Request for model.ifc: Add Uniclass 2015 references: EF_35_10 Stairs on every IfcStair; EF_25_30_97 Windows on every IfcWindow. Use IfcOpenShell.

First a look at what the model holds.

```python
import ifcopenshell

model = ifcopenshell.open("model.ifc")
print(model.schema)
print("classifications:", [c.Name for c in model.by_type("IfcClassification")])
for ifc_class in ("IfcDoor", "IfcRoof", "IfcStair", "IfcWall", "IfcWindow"):
    print(ifc_class, len(model.by_type(ifc_class)))
```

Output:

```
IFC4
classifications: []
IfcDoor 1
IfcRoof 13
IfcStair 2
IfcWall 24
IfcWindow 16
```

```python
import ifcopenshell
import ifcopenshell.api.classification

model = ifcopenshell.open("model.ifc")

system = ifcopenshell.api.classification.add_classification(model, classification="Uniclass 2015")

codes = {
    "IfcStair": ("EF_35_10", "Stairs"),
    "IfcWindow": ("EF_25_30_97", "Windows"),
}
for ifc_class, (code, name) in codes.items():
    products = model.by_type(ifc_class)
    ifcopenshell.api.classification.add_reference(
        model, products=products, classification=system, identification=code, name=name
    )
    print(code, len(products))

model.write("model_edited.ifc")
```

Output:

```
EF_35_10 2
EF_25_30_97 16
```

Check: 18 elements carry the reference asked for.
